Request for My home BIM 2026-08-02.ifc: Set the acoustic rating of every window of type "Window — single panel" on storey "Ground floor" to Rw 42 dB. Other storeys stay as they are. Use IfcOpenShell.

First a look at what the model holds.

```python
import ifcopenshell
import ifcopenshell.util.element

model = ifcopenshell.open("My home BIM 2026-08-02.ifc")
print(model.schema)
storey = next(s for s in model.by_type("IfcBuildingStorey") if s.Name == "Ground floor")
windows = [e for e in ifcopenshell.util.element.get_decomposition(storey) if e.is_a("IfcWindow")]
seen = {}
for e in windows:
    element_type = ifcopenshell.util.element.get_type(e)
    key = (element_type.Name if element_type != e and element_type else None, ifcopenshell.util.element.get_pset(e, "Pset_WindowCommon", "AcousticRating"))
    seen[key] = seen.get(key, 0) + 1
for (name, value), count in sorted(seen.items(), key=str):
    print(count, "x", name, "|", value)
```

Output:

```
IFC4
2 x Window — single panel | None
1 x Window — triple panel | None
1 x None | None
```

```python
import ifcopenshell
import ifcopenshell.api.pset
import ifcopenshell.util.element

model = ifcopenshell.open("My home BIM 2026-08-02.ifc")

storey = next(s for s in model.by_type("IfcBuildingStorey") if s.Name == "Ground floor")
windows = [e for e in ifcopenshell.util.element.get_decomposition(storey) if e.is_a("IfcWindow")]

count = 0
for e in windows:
    element_type = ifcopenshell.util.element.get_type(e)
    if element_type in (None, e) or element_type.Name != "Window — single panel":
        continue
    # add_pset returns the element's existing set when there is one.
    pset = ifcopenshell.api.pset.add_pset(model, product=e, name="Pset_WindowCommon")
    ifcopenshell.api.pset.edit_pset(model, pset=pset, properties={"AcousticRating": "Rw 42 dB"})
    count += 1

print(count, "windows updated")

model.write("My home BIM 2026-08-02_v2.ifc")
```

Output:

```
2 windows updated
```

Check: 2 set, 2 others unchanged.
